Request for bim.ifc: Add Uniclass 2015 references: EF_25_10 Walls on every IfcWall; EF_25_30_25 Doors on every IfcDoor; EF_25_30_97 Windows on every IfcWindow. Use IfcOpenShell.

First a look at what the model holds.

```python
import ifcopenshell

model = ifcopenshell.open("bim.ifc")
print(model.schema)
print("classifications:", [c.Name for c in model.by_type("IfcClassification")])
for ifc_class in ("IfcDoor", "IfcRoof", "IfcStair", "IfcWall", "IfcWindow"):
    print(ifc_class, len(model.by_type(ifc_class)))
```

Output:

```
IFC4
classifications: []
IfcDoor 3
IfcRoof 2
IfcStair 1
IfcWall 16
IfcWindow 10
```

```python
import ifcopenshell
import ifcopenshell.api.classification

model = ifcopenshell.open("bim.ifc")

system = ifcopenshell.api.classification.add_classification(model, classification="Uniclass 2015")

codes = {
    "IfcWall": ("EF_25_10", "Walls"),
    "IfcDoor": ("EF_25_30_25", "Doors"),
    "IfcWindow": ("EF_25_30_97", "Windows"),
}
for ifc_class, (code, name) in codes.items():
    products = model.by_type(ifc_class)
    ifcopenshell.api.classification.add_reference(
        model, products=products, classification=system, identification=code, name=name
    )
    print(code, len(products))

model.write("bim-out.ifc")
```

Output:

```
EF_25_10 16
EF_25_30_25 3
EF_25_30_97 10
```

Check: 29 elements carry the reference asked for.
